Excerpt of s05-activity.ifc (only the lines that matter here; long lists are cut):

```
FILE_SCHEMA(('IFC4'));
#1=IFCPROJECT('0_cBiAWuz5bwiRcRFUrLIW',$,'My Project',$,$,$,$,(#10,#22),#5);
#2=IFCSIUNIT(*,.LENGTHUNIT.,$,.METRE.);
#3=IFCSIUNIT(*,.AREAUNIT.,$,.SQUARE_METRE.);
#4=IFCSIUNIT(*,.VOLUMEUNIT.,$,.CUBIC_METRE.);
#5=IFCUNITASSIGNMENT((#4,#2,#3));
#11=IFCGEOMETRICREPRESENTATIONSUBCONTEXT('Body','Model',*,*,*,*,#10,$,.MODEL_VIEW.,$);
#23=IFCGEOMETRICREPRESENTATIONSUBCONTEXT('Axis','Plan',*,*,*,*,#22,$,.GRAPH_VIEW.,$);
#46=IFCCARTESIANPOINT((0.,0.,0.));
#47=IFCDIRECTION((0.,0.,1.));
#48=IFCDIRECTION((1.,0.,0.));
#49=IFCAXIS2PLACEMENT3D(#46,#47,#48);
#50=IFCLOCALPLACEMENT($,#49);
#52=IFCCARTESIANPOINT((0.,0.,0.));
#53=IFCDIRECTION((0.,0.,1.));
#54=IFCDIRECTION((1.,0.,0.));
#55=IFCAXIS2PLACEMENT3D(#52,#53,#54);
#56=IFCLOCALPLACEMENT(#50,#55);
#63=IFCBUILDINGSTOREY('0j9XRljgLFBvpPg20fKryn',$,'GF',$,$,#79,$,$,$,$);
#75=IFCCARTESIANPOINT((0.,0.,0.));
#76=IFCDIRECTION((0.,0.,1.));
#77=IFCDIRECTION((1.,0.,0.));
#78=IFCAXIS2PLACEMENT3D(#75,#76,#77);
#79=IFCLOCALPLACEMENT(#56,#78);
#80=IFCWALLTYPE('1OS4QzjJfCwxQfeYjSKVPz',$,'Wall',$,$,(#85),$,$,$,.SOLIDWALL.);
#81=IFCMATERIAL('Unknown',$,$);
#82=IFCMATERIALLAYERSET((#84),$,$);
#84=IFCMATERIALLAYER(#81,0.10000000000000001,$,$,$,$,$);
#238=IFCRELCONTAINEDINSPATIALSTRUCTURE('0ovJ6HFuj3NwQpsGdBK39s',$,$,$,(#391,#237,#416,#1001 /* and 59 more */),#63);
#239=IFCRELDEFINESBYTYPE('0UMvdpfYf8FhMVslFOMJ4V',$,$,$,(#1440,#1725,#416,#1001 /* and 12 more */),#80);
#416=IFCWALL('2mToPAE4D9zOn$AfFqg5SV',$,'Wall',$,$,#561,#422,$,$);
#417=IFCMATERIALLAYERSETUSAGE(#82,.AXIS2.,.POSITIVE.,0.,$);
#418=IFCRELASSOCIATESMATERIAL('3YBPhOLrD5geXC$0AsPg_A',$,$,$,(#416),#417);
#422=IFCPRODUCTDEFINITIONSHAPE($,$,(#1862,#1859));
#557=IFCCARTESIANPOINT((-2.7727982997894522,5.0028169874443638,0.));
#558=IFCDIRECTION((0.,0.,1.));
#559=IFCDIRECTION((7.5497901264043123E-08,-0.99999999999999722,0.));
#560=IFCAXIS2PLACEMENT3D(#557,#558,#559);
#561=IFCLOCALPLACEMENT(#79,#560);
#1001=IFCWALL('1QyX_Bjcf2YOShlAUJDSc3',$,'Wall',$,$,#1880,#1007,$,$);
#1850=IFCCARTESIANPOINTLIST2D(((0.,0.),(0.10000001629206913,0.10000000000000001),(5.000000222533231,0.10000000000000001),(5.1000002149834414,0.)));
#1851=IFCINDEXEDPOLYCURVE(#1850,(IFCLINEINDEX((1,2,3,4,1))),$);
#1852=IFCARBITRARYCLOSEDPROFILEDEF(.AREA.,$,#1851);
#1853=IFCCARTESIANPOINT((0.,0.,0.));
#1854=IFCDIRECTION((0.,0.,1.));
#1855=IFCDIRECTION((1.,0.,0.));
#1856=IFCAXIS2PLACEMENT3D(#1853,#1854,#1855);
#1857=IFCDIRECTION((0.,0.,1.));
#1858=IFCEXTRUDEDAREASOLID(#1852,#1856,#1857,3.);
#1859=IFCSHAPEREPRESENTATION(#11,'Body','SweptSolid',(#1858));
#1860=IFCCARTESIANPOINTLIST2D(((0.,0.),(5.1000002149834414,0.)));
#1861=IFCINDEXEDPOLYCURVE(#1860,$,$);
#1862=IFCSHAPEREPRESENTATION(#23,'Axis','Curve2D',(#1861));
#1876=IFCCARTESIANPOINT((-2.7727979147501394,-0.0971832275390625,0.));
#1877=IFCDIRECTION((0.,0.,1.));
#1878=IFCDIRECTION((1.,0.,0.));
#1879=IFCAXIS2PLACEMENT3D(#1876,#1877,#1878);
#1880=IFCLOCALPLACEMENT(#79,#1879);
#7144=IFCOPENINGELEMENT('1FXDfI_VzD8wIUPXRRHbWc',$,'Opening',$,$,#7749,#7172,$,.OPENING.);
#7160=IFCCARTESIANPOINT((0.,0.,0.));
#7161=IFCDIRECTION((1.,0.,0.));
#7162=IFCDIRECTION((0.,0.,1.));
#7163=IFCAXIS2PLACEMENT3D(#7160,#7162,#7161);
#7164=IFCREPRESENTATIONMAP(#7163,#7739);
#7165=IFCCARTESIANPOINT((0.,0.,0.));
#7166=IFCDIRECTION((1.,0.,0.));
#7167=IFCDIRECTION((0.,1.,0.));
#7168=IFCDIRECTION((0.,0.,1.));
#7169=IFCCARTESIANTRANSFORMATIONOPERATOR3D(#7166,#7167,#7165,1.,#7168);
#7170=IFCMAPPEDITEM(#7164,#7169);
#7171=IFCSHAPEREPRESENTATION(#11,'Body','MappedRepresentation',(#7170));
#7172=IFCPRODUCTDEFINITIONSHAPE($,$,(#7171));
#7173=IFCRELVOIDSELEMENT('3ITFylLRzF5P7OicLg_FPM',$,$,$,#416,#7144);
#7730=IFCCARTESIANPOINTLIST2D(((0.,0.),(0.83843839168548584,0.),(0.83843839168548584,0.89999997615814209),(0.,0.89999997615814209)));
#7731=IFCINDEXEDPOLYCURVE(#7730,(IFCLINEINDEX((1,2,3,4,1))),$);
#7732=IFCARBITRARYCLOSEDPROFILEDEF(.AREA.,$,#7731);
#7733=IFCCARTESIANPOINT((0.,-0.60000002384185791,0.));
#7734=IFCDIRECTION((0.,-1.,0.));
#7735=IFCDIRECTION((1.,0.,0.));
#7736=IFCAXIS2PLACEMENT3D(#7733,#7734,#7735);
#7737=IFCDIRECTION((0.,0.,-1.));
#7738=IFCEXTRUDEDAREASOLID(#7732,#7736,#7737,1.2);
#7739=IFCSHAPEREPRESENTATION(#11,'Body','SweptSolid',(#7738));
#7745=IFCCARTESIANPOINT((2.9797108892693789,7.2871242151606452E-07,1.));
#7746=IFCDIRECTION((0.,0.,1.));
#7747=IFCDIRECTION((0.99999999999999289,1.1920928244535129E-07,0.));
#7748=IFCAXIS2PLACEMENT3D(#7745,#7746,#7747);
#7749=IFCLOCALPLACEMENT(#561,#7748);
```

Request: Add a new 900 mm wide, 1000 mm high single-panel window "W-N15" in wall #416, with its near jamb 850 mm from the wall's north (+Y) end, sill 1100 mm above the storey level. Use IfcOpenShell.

```python
import numpy as np
import ifcopenshell
import ifcopenshell.api.feature
import ifcopenshell.api.geometry
import ifcopenshell.api.root
import ifcopenshell.api.spatial
import ifcopenshell.geom
import ifcopenshell.util.element
import ifcopenshell.util.placement
import ifcopenshell.util.representation
import ifcopenshell.util.shape
import ifcopenshell.util.unit

model = ifcopenshell.open("s05-activity.ifc")
unit_scale = ifcopenshell.util.unit.calculate_unit_scale(model)
settings = ifcopenshell.geom.settings()


def volume(element):
    """Net volume in cubic metres, openings subtracted."""
    shape = ifcopenshell.geom.create_shape(settings, element)
    return ifcopenshell.util.shape.get_volume(shape.geometry)


wall = model.by_guid("2mToPAE4D9zOn$AfFqg5SV")
storey = ifcopenshell.util.element.get_container(wall, ifc_class="IfcBuildingStorey")
context = ifcopenshell.util.representation.get_context(model, "Model", "Body", "MODEL_VIEW")
before = volume(wall)

width, height, from_end, sill = 0.9, 1, 0.85, 1.1  # metres

# The wall runs along its own X axis, and the end named is its -X end.
wall_shape = ifcopenshell.geom.create_shape(settings, wall)
x, y, z = ifcopenshell.util.shape.get_vertices(wall_shape.geometry).T
start = x.min() + from_end
face, thickness = float(y.min()), float(y.max() - y.min())
wall_matrix = ifcopenshell.util.placement.get_local_placement(wall.ObjectPlacement)
level = ifcopenshell.util.placement.get_local_placement(storey.ObjectPlacement)[2, 3]


def in_wall(x, y):
    """Placement at x, y metres in the wall's axes, at sill height."""
    matrix = wall_matrix.copy()
    matrix[:, 3] = wall_matrix @ np.array([x / unit_scale, y / unit_scale, 0.0, 1.0])
    matrix[2, 3] = level + sill / unit_scale
    return matrix


# Opening: a box that overshoots both wall faces by 50 mm.
opening = ifcopenshell.api.root.create_entity(model, ifc_class="IfcOpeningElement", predefined_type="OPENING")
box = ifcopenshell.api.geometry.add_wall_representation(
    model, context=context, length=width, height=height, thickness=thickness + 0.1
)
ifcopenshell.api.geometry.assign_representation(model, product=opening, representation=box)
ifcopenshell.api.geometry.edit_object_placement(model, product=opening, matrix=in_wall(start, face - 0.05), is_si=False)
ifcopenshell.api.feature.add_feature(model, feature=opening, element=wall)

window = ifcopenshell.api.root.create_entity(model, ifc_class="IfcWindow", name="W-N15", predefined_type="WINDOW")
window.OverallWidth, window.OverallHeight = width / unit_scale, height / unit_scale
window.PartitioningType = "SINGLE_PANEL"
body = ifcopenshell.api.geometry.add_window_representation(
    model,
    context=context,
    overall_width=window.OverallWidth,
    overall_height=window.OverallHeight,
    partition_type="SINGLE_PANEL",
)
ifcopenshell.api.geometry.assign_representation(model, product=window, representation=body)
ifcopenshell.api.spatial.assign_container(model, products=[window], relating_structure=storey)
ifcopenshell.api.feature.add_filling(model, opening=opening, element=window)

# Centre the window in the wall's thickness.
ifcopenshell.api.geometry.edit_object_placement(model, product=window, matrix=in_wall(start, face), is_si=False)
window_shape = ifcopenshell.geom.create_shape(settings, window)
depth = ifcopenshell.util.shape.get_vertices(window_shape.geometry)[:, 1]
offset = face + thickness / 2 - (depth.min() + depth.max()) / 2
ifcopenshell.api.geometry.edit_object_placement(model, product=window, matrix=in_wall(start, offset), is_si=False)

after = volume(wall)

print(f"wall volume {before:.3f} -> {after:.3f} m3")

model.write("s05-activity_updated.ifc")
```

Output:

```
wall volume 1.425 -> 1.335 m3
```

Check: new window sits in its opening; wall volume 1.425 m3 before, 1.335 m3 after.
